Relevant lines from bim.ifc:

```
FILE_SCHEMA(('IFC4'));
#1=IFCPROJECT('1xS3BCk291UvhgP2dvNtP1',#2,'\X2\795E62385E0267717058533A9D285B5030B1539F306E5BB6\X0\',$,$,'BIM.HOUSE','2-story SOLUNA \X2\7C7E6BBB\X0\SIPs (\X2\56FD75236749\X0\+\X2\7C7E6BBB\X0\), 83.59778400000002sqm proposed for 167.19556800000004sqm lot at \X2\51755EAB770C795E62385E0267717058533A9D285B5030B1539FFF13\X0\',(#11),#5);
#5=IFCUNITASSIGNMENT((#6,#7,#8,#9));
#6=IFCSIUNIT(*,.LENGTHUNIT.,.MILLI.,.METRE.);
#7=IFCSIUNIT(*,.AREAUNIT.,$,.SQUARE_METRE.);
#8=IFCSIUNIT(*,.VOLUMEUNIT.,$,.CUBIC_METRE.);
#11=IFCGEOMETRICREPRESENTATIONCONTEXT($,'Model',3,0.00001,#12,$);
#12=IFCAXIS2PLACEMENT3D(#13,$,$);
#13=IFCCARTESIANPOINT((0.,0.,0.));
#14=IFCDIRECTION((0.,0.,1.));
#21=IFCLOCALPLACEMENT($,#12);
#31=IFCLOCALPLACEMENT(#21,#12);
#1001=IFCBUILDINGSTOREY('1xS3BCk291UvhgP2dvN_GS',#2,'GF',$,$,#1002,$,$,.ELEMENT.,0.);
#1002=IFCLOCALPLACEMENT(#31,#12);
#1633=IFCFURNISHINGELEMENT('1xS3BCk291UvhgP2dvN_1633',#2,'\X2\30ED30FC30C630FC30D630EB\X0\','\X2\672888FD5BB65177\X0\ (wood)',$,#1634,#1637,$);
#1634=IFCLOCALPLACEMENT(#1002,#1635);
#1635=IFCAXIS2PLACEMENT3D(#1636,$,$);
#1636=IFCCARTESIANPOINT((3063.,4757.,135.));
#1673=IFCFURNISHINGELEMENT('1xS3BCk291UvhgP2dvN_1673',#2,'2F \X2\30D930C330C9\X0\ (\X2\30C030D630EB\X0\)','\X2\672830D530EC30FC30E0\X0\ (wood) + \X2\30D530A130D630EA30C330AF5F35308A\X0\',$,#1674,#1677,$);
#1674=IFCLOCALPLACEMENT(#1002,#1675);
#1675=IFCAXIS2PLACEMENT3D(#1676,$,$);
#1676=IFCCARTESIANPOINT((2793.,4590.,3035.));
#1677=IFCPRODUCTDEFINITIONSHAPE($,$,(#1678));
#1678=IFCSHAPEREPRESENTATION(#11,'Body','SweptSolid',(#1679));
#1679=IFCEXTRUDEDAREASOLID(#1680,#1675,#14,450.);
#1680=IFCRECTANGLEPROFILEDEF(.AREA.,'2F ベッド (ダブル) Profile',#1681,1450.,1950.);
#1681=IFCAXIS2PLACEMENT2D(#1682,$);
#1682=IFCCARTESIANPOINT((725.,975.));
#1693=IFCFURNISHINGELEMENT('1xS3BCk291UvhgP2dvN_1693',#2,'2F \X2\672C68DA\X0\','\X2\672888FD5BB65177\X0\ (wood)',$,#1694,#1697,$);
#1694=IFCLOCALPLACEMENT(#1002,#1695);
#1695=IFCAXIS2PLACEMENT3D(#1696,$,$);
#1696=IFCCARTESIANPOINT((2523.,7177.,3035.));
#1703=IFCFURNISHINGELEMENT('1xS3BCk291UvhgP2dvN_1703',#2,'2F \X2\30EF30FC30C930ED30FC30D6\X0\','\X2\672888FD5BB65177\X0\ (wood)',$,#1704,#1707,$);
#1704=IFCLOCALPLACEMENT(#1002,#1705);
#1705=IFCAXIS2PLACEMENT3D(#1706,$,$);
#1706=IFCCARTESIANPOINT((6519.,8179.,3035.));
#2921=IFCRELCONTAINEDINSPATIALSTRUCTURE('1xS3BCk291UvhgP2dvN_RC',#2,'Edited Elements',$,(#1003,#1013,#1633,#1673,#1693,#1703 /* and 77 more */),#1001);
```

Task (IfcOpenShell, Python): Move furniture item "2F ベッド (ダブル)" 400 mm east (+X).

```python
import ifcopenshell
import ifcopenshell.api.geometry
import ifcopenshell.util.placement
import ifcopenshell.util.unit

model = ifcopenshell.open("bim.ifc")
unit_scale = ifcopenshell.util.unit.calculate_unit_scale(model)

item = model.by_guid("1xS3BCk291UvhgP2dvN_1673")
matrix = ifcopenshell.util.placement.get_local_placement(item.ObjectPlacement)
matrix[0, 3] += 0.4 / unit_scale
ifcopenshell.api.geometry.edit_object_placement(model, product=item, matrix=matrix, is_si=False)

print(ifcopenshell.util.placement.get_local_placement(item.ObjectPlacement).round(3) + 0.0)

model.write("bim_edited.ifc")
```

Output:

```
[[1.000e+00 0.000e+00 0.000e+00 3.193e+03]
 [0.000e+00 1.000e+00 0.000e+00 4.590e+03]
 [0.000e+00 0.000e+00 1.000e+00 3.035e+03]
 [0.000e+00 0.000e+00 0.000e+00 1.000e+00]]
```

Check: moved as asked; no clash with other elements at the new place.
